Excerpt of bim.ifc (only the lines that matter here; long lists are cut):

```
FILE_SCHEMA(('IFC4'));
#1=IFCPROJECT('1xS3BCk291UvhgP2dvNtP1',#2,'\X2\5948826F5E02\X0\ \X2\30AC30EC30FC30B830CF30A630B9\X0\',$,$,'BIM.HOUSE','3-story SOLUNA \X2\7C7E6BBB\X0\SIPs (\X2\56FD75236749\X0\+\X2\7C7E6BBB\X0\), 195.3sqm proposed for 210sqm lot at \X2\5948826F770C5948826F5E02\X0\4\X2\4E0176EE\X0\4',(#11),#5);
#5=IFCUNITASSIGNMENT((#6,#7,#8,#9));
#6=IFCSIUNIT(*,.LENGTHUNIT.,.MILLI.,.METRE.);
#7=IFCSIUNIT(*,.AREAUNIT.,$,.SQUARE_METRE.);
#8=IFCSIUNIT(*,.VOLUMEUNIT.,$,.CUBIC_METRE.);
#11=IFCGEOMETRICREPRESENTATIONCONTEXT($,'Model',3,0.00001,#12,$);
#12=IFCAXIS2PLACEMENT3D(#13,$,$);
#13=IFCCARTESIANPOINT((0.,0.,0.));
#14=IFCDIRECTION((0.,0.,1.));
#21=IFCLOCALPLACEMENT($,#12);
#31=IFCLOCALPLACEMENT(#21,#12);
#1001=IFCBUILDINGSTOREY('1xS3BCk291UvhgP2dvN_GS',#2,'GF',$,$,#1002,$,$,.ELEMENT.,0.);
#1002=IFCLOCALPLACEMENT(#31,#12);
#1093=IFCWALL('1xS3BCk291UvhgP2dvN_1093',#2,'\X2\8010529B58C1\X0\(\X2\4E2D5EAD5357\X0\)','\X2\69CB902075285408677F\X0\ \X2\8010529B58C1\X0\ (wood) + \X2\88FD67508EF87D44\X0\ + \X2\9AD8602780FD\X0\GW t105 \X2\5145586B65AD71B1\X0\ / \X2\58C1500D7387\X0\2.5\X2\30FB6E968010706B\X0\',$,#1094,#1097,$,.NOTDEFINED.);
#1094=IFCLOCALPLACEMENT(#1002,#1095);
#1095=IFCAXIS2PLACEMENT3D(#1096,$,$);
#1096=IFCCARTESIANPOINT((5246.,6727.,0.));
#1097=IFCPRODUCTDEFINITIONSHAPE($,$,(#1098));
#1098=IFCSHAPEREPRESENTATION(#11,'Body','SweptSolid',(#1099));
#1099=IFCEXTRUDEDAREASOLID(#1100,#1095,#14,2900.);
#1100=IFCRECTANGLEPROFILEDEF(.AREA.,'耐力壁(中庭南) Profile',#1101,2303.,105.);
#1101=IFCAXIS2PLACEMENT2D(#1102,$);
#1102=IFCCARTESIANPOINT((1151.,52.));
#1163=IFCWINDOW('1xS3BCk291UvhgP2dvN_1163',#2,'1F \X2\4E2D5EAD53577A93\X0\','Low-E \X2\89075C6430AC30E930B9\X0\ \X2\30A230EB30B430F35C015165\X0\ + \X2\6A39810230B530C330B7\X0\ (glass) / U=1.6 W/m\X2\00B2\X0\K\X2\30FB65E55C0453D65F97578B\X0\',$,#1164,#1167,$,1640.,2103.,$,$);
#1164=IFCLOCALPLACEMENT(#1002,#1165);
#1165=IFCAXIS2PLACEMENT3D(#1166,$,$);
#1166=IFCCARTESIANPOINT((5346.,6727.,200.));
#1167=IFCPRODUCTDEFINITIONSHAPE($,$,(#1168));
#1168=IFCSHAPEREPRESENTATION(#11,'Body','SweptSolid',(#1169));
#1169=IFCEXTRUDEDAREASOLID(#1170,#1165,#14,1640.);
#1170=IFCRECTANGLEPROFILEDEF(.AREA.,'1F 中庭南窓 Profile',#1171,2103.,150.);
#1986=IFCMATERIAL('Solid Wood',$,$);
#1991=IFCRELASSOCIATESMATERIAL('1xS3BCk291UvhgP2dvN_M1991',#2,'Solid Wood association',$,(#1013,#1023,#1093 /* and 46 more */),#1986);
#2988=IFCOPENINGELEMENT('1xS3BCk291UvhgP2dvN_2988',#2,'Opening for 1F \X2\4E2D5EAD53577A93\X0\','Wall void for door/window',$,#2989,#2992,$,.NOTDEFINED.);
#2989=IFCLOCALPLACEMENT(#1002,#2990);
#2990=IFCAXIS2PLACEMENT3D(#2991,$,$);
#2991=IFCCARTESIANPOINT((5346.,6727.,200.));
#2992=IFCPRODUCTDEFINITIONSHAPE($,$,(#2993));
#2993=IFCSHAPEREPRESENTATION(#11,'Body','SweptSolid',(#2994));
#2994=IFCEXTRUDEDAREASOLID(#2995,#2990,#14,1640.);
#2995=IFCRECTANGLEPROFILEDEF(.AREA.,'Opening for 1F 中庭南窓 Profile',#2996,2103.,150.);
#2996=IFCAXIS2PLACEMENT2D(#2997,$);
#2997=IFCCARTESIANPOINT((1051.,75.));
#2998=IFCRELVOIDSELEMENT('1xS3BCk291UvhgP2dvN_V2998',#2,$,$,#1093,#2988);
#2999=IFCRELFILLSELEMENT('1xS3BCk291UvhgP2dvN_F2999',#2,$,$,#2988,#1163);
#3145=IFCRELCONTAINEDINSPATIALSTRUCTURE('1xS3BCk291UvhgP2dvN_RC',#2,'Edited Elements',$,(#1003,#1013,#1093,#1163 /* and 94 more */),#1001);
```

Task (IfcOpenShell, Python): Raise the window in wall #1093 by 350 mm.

```python
import numpy as np
import ifcopenshell
import ifcopenshell.api.geometry
import ifcopenshell.util.placement
import ifcopenshell.util.unit

model = ifcopenshell.open("bim.ifc")
unit_scale = ifcopenshell.util.unit.calculate_unit_scale(model)

window = model.by_guid("1xS3BCk291UvhgP2dvN_1163")
opening = window.FillsVoids[0].RelatingOpeningElement
dz = 0.35 / unit_scale

shift = np.array([0.0, 0.0, dz])
# The window is not placed relative to its opening, so move both.
for product in (opening, window):
    matrix = ifcopenshell.util.placement.get_local_placement(product.ObjectPlacement)
    matrix[:3, 3] += shift
    ifcopenshell.api.geometry.edit_object_placement(model, product=product, matrix=matrix, is_si=False)

print(f"moved by {dz * unit_scale:+.3f} m")

model.write("bim-out.ifc")
```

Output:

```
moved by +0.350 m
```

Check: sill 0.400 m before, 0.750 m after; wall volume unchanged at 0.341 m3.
